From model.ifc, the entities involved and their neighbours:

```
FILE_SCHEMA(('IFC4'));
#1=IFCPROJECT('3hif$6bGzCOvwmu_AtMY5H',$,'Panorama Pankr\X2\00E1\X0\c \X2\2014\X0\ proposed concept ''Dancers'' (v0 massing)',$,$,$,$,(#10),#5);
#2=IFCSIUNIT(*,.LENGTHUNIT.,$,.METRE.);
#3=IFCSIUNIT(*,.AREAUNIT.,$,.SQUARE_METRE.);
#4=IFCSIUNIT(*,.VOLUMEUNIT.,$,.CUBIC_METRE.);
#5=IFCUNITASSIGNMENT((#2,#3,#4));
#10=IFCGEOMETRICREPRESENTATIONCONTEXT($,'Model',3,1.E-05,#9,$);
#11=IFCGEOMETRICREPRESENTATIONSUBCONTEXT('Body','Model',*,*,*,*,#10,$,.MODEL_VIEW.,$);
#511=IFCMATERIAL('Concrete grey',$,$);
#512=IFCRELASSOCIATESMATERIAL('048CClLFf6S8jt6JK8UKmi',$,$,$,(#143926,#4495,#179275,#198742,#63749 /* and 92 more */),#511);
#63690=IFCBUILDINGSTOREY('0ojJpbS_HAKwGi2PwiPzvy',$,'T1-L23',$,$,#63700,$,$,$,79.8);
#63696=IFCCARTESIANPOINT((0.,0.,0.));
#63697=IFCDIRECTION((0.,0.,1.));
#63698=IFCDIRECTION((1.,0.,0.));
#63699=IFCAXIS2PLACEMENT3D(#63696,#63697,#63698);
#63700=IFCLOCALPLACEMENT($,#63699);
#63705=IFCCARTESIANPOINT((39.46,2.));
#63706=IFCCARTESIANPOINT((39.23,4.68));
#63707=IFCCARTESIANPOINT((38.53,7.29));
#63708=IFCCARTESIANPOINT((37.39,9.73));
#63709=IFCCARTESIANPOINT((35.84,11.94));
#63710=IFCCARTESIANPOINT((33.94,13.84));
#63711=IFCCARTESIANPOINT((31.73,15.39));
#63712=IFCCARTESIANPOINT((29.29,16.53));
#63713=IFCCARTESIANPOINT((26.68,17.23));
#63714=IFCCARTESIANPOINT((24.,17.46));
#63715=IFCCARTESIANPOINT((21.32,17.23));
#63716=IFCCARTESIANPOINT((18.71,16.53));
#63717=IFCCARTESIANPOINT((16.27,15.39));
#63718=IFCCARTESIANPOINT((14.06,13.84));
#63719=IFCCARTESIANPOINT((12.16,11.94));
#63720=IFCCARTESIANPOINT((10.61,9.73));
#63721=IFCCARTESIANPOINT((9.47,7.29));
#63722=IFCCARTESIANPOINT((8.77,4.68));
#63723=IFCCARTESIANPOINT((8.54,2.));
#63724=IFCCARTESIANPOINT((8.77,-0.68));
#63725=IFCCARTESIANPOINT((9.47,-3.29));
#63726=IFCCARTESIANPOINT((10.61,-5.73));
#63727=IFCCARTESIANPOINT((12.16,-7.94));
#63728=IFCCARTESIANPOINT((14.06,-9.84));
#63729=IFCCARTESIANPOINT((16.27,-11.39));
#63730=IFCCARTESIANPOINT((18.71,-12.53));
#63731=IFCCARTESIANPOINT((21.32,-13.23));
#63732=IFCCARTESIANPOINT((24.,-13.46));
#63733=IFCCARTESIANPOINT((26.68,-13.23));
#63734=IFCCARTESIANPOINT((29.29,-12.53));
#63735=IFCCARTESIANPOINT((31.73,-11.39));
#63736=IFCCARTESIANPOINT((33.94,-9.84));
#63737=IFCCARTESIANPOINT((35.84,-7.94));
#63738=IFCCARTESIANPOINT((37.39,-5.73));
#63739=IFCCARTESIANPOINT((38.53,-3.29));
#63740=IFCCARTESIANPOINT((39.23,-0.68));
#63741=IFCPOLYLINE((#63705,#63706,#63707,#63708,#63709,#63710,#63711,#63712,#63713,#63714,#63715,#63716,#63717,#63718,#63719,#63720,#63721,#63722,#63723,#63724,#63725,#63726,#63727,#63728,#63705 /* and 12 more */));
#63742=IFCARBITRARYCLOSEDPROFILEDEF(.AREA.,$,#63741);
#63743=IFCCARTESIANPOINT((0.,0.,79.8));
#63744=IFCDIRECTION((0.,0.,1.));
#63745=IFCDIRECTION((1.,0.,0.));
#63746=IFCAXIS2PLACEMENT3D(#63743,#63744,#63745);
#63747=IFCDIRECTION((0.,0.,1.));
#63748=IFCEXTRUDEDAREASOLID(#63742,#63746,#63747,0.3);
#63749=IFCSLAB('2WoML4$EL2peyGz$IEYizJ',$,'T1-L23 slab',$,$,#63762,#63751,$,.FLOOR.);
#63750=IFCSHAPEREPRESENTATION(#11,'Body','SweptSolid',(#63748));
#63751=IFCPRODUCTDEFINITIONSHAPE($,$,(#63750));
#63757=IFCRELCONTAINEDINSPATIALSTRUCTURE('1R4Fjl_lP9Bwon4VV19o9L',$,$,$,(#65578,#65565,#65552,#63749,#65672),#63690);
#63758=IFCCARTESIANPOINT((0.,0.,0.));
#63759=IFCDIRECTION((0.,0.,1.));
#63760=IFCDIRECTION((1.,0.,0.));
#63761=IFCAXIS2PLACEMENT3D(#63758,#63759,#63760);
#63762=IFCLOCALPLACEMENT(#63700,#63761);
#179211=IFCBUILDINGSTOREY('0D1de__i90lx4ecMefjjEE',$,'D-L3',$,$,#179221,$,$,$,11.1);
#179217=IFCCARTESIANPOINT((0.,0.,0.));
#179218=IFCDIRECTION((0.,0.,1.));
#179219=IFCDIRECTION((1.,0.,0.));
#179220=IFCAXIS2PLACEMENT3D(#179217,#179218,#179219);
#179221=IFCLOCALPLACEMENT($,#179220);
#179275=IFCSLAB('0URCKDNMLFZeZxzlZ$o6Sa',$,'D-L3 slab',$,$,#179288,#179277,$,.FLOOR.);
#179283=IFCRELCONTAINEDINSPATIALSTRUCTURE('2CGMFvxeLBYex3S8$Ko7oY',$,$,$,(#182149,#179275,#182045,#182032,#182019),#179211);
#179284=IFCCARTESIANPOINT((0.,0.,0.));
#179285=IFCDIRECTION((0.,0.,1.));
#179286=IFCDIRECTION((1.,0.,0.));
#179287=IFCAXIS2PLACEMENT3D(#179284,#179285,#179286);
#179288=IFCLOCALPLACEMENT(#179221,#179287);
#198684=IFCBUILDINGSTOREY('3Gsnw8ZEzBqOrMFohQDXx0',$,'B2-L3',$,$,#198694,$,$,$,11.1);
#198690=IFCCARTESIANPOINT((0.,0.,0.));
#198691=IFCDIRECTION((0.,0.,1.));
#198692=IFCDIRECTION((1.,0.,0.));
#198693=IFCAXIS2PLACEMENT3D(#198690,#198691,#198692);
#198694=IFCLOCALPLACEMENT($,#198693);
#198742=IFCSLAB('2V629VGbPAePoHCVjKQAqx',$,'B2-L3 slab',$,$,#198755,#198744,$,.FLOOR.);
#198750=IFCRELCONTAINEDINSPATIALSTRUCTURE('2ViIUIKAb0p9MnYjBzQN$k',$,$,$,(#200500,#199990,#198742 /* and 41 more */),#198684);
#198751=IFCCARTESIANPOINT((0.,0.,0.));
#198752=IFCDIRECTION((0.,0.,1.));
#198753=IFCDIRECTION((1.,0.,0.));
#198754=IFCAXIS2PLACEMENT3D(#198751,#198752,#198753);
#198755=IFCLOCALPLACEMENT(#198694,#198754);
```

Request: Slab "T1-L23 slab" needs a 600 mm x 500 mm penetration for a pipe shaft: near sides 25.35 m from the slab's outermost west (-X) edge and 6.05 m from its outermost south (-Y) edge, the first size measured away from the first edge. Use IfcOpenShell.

```python
import numpy as np
import ifcopenshell
import ifcopenshell.api.feature
import ifcopenshell.api.geometry
import ifcopenshell.api.root
import ifcopenshell.geom
import ifcopenshell.util.placement
import ifcopenshell.util.representation
import ifcopenshell.util.shape
import ifcopenshell.util.unit

model = ifcopenshell.open("model.ifc")
unit_scale = ifcopenshell.util.unit.calculate_unit_scale(model)
settings = ifcopenshell.geom.settings()


def volume(element):
    """Net volume in cubic metres, openings subtracted."""
    shape = ifcopenshell.geom.create_shape(settings, element)
    return ifcopenshell.util.shape.get_volume(shape.geometry)


slab = model.by_guid("2WoML4$EL2peyGz$IEYizJ")
before = volume(slab)

# Extent in the slab's own axes, in metres. The edges named are its -X and -Y sides.
slab_shape = ifcopenshell.geom.create_shape(settings, slab)
vertices = ifcopenshell.util.shape.get_vertices(slab_shape.geometry)
x_min, y_min, bottom = vertices.min(axis=0)
top = vertices[:, 2].max()

opening = ifcopenshell.api.root.create_entity(model, ifc_class="IfcOpeningElement", name="Pipe shaft opening", predefined_type="OPENING")
context = ifcopenshell.util.representation.get_context(model, "Model", "Body", "MODEL_VIEW")
width, depth = 0.6, 0.5
outline = [(0.0, 0.0), (width, 0.0), (width, depth), (0.0, depth), (0.0, 0.0)]
# Overshoot both faces by 50 mm so the cut is clean.
shape = ifcopenshell.api.geometry.add_slab_representation(
    model, context=context, depth=top - bottom + 0.1, polyline=outline
)
ifcopenshell.api.geometry.assign_representation(model, product=opening, representation=shape)

matrix = ifcopenshell.util.placement.get_local_placement(slab.ObjectPlacement)
matrix[:, 3] = matrix @ np.append(np.array([x_min + 25.35, y_min + 6.05, bottom - 0.05]) / unit_scale, 1.0)
ifcopenshell.api.geometry.edit_object_placement(model, product=opening, matrix=matrix, is_si=False)
ifcopenshell.api.feature.add_feature(model, feature=opening, element=slab)

after = volume(slab)

print(f"slab volume {before:.3f} -> {after:.3f} m3")

model.write("model_updated.ifc")
```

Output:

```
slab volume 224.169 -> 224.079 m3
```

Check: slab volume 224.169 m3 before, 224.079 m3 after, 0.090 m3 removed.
